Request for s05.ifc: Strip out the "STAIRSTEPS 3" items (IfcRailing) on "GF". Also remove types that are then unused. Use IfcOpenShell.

First a look at what the model holds.

```python
import ifcopenshell
import ifcopenshell.util.element

model = ifcopenshell.open("s05.ifc")
print(model.schema)
storey = next(s for s in model.by_type("IfcBuildingStorey") if s.Name == "GF")
railings = [e for e in ifcopenshell.util.element.get_decomposition(storey) if e.is_a("IfcRailing")]
seen = {}
for e in railings:
    element_type = ifcopenshell.util.element.get_type(e)
    name = element_type.Name if element_type not in (None, e) else None
    seen[name] = seen.get(name, 0) + 1
for name, count in sorted(seen.items(), key=str):
    print(count, "x", name)
```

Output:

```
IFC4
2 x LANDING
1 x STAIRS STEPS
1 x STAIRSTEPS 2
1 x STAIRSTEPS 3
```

```python
import ifcopenshell
import ifcopenshell.api.root
import ifcopenshell.util.element

model = ifcopenshell.open("s05.ifc")

storey = next(s for s in model.by_type("IfcBuildingStorey") if s.Name == "GF")
railings = [e for e in ifcopenshell.util.element.get_decomposition(storey) if e.is_a("IfcRailing")]
targets = [e for e in railings if (t := ifcopenshell.util.element.get_type(e)) not in (None, e) and t.Name == "STAIRSTEPS 3"]
types = {ifcopenshell.util.element.get_type(e) for e in targets} - {None, *targets}

for e in targets:
    ifcopenshell.api.root.remove_product(model, product=e)
print(len(targets), "removed")

unused = [t for t in types if not ifcopenshell.util.element.get_types(t)]
for t in unused:
    ifcopenshell.api.root.remove_product(model, product=t)
print(len(unused), "unused types removed")

model.write("s05_updated.ifc")
```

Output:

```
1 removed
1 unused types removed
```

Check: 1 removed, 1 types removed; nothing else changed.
